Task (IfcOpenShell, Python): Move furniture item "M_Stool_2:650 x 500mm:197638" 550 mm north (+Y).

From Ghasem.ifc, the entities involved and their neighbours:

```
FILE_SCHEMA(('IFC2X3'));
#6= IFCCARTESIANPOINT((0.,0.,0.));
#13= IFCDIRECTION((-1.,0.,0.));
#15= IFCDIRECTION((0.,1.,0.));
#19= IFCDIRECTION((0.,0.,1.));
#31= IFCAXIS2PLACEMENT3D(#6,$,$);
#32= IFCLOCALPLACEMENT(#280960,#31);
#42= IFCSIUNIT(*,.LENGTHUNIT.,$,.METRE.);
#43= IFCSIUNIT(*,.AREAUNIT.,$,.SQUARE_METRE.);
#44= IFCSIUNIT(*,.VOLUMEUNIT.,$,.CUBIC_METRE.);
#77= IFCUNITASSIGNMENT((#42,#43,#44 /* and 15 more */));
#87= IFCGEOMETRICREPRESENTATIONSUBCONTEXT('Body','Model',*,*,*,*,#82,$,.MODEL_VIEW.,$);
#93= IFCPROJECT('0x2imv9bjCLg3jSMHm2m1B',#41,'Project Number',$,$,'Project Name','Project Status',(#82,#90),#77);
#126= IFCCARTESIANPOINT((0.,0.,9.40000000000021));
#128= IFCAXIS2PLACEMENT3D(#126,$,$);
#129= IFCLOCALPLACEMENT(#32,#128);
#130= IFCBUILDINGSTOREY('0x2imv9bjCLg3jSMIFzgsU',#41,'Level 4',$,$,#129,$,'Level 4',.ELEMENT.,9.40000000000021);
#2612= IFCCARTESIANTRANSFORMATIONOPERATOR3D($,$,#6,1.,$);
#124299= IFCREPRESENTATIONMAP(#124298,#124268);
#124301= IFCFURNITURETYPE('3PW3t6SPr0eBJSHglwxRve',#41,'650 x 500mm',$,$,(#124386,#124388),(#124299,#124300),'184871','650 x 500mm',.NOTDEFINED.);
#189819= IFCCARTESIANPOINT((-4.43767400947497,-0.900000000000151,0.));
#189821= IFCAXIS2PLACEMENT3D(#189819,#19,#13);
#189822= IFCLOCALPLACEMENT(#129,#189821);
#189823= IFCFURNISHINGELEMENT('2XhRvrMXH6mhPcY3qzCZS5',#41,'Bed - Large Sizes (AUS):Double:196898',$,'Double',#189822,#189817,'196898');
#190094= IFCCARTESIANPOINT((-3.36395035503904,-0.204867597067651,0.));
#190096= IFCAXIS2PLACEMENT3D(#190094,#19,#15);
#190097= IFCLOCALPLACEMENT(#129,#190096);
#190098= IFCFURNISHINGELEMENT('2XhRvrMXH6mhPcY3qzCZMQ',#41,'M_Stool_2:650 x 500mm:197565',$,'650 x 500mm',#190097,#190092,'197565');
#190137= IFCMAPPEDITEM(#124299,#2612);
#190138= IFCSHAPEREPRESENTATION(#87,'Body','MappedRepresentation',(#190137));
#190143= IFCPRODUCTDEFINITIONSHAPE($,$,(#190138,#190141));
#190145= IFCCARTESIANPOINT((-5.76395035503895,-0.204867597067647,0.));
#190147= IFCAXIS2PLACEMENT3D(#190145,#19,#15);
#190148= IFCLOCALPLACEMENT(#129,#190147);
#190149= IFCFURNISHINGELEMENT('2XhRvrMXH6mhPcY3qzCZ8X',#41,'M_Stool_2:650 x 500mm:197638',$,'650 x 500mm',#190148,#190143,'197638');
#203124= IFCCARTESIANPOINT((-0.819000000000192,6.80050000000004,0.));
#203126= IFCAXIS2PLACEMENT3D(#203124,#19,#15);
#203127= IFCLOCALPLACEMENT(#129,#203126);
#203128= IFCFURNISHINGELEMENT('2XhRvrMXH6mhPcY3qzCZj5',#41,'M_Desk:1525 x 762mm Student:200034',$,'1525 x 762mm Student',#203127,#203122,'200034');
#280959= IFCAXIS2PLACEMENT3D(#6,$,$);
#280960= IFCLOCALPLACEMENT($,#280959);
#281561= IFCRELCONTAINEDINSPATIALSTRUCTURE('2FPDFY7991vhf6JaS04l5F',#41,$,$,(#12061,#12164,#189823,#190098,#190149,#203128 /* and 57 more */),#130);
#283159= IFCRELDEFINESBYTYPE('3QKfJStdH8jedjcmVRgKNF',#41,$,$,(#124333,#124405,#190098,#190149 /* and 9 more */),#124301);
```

```python
import ifcopenshell
import ifcopenshell.api.geometry
import ifcopenshell.util.placement
import ifcopenshell.util.unit

model = ifcopenshell.open("Ghasem.ifc")
unit_scale = ifcopenshell.util.unit.calculate_unit_scale(model)

item = model.by_guid("2XhRvrMXH6mhPcY3qzCZ8X")
matrix = ifcopenshell.util.placement.get_local_placement(item.ObjectPlacement)
matrix[1, 3] += 0.55 / unit_scale
ifcopenshell.api.geometry.edit_object_placement(model, product=item, matrix=matrix, is_si=False)

print(ifcopenshell.util.placement.get_local_placement(item.ObjectPlacement).round(3) + 0.0)

model.write("Ghasem-out.ifc")
```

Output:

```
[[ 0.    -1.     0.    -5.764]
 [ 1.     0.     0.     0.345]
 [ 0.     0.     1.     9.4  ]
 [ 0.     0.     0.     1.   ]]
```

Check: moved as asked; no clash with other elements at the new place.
